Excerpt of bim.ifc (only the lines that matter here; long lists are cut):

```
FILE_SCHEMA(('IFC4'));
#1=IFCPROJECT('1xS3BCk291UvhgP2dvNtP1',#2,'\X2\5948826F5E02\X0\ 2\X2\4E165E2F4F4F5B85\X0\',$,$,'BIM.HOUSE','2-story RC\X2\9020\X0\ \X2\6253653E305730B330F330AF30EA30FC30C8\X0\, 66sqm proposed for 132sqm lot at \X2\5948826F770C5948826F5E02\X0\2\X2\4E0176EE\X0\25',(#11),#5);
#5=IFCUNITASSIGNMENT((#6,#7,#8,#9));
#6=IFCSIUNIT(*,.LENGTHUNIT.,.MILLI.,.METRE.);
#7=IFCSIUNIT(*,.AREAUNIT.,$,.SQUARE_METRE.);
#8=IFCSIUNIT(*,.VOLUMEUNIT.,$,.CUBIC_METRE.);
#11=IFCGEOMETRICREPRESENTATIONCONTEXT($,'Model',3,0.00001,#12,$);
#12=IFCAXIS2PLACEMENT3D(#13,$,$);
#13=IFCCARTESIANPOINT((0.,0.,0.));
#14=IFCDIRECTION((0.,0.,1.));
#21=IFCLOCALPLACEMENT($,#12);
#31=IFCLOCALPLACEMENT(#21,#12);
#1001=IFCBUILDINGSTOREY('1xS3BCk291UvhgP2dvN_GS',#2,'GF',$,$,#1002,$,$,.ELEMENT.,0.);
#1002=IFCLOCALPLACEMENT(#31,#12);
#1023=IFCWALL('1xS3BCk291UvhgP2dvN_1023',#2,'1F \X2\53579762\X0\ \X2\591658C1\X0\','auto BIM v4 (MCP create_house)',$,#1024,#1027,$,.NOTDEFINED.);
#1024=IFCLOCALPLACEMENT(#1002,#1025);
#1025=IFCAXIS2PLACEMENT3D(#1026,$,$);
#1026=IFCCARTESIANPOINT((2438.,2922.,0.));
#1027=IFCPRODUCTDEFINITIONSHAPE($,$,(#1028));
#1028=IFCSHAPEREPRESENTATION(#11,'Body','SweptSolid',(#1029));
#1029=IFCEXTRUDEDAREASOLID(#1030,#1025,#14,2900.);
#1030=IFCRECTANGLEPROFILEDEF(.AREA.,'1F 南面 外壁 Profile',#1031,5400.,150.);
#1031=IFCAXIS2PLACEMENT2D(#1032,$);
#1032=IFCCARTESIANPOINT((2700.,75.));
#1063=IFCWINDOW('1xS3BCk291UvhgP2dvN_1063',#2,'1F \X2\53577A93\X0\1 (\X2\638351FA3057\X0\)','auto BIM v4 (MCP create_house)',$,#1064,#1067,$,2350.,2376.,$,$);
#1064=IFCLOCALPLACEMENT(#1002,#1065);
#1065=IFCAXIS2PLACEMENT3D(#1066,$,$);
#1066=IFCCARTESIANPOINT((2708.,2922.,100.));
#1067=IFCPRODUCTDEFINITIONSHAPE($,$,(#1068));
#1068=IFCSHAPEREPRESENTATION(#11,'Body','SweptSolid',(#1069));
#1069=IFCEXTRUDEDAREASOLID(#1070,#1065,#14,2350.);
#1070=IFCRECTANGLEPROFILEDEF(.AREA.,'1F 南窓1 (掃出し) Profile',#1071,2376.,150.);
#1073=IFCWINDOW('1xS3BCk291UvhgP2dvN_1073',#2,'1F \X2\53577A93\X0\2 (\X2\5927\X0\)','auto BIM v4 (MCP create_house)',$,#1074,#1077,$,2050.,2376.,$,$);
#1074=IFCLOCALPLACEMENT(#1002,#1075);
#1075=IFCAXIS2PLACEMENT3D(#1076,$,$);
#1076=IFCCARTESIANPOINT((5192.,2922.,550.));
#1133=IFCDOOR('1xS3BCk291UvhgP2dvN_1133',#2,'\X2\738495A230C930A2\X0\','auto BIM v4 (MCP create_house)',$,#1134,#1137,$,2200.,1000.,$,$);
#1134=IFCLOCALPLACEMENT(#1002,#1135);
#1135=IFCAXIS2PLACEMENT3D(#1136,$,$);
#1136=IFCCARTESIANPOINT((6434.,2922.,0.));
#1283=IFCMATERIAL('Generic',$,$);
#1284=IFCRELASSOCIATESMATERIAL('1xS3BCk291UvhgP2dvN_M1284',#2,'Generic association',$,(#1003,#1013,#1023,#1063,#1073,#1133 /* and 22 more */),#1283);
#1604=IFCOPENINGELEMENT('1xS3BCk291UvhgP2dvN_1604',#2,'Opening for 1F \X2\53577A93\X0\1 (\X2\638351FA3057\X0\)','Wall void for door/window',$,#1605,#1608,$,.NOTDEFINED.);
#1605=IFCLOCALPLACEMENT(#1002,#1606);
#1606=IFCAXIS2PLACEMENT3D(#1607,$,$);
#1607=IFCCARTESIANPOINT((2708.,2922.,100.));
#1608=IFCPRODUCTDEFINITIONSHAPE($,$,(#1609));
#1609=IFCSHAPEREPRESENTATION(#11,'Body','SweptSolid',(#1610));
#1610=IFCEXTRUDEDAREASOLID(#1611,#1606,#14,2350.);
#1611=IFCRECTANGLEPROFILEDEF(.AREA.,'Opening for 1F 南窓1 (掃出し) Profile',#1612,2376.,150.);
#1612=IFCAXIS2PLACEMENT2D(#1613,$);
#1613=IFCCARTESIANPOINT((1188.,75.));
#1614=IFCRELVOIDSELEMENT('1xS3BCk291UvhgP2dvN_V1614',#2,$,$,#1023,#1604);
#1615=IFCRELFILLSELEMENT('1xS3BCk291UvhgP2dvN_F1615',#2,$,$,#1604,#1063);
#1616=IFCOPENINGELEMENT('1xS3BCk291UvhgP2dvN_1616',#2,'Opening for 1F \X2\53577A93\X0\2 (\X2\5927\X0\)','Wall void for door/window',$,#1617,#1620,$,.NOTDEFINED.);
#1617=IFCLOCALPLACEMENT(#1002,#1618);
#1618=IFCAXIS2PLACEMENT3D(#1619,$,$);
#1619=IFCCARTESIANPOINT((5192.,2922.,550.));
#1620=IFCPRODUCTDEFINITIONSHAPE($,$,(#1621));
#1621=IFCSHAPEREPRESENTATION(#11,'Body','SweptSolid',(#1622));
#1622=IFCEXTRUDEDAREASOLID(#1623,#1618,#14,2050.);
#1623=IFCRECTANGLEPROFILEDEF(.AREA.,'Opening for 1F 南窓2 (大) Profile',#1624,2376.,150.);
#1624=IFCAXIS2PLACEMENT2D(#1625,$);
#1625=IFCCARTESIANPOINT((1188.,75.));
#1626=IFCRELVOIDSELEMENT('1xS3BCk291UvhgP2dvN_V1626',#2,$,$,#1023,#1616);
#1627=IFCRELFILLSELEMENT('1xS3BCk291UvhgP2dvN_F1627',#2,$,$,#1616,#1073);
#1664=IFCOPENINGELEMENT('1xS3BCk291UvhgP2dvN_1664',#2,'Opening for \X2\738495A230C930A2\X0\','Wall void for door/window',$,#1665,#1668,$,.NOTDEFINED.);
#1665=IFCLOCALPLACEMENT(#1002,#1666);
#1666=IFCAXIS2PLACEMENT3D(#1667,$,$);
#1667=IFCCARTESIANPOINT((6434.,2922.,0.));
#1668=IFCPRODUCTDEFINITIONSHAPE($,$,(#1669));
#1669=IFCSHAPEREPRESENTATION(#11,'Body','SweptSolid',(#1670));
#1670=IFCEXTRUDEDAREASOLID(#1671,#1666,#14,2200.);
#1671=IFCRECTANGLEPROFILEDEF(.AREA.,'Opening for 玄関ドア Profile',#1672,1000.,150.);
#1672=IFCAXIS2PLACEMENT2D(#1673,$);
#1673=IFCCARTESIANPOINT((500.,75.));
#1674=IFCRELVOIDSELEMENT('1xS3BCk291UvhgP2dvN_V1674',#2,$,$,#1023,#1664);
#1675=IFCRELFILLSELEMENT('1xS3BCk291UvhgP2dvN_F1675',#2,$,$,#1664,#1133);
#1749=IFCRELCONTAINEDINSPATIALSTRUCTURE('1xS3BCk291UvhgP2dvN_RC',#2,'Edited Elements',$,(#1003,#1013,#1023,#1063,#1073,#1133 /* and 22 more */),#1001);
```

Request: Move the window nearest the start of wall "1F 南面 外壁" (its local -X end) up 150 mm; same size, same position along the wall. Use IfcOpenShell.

```python
import numpy as np
import ifcopenshell
import ifcopenshell.api.geometry
import ifcopenshell.util.placement
import ifcopenshell.util.unit

model = ifcopenshell.open("bim.ifc")
unit_scale = ifcopenshell.util.unit.calculate_unit_scale(model)

window = model.by_guid("1xS3BCk291UvhgP2dvN_1063")
opening = window.FillsVoids[0].RelatingOpeningElement
dz = 150.0

shift = np.array([0.0, 0.0, dz])
# The window is not placed relative to its opening, so move both.
for product in (opening, window):
    matrix = ifcopenshell.util.placement.get_local_placement(product.ObjectPlacement)
    matrix[:3, 3] += shift
    ifcopenshell.api.geometry.edit_object_placement(model, product=product, matrix=matrix, is_si=False)

print(f"moved by {dz * unit_scale:+.3f} m")

model.write("bim_rev.ifc")
```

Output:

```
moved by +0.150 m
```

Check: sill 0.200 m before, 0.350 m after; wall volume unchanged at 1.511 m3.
